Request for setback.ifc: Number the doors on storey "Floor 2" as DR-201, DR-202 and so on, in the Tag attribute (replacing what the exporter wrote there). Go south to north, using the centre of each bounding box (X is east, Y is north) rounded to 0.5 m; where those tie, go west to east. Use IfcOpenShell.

First a look at what the model holds.

```python
import ifcopenshell
import ifcopenshell.util.element
import ifcopenshell.util.placement

model = ifcopenshell.open("setback.ifc")
print(model.schema)
storey = next(s for s in model.by_type("IfcBuildingStorey") if s.Name == "Floor 2")
doors = [e for e in ifcopenshell.util.element.get_decomposition(storey) if e.is_a("IfcDoor")]
for e in sorted(doors, key=lambda e: e.id()):
    origin = ifcopenshell.util.placement.get_local_placement(e.ObjectPlacement)[:3, 3]
    print(e.id(), e.Tag, e.Name, origin.round(2) + 0.0, sep=" | ")
```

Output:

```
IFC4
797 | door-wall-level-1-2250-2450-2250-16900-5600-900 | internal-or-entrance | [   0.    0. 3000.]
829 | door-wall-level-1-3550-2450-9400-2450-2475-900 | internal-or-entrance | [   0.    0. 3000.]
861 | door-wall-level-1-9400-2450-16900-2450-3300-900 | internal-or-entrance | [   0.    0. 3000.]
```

```python
import ifcopenshell
import ifcopenshell.geom
import ifcopenshell.util.element
import ifcopenshell.util.shape

model = ifcopenshell.open("setback.ifc")
settings = ifcopenshell.geom.settings()
settings.set("use-world-coords", True)


def centre(element):
    shape = ifcopenshell.geom.create_shape(settings, element)
    return ifcopenshell.util.shape.get_bbox_centroid(shape.geometry)


storey = next(s for s in model.by_type("IfcBuildingStorey") if s.Name == "Floor 2")
doors = [e for e in ifcopenshell.util.element.get_decomposition(storey) if e.is_a("IfcDoor")]

# Insertion points can sit at a corner or the storey origin, so sort by the geometry (in metres).
centres = {e: centre(e) for e in doors}
doors.sort(key=lambda e: (round(centres[e][1] / 0.5), centres[e][0]))

for i, e in enumerate(doors, start=1):
    number = f"DR-2{i:02d}"
    e.Tag = number
    print(e.id(), number)

model.write("setback_rev.ifc")
```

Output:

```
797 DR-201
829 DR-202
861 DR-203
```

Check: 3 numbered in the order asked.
